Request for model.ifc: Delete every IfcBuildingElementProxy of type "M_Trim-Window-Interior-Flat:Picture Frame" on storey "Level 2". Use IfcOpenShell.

First a look at what the model holds.

```python
import ifcopenshell
import ifcopenshell.util.element

model = ifcopenshell.open("model.ifc")
print(model.schema)
storey = next(s for s in model.by_type("IfcBuildingStorey") if s.Name == "Level 2")
proxies = [e for e in ifcopenshell.util.element.get_decomposition(storey) if e.is_a("IfcBuildingElementProxy")]
seen = {}
for e in proxies:
    element_type = ifcopenshell.util.element.get_type(e)
    name = element_type.Name if element_type not in (None, e) else None
    seen[name] = seen.get(name, 0) + 1
for name, count in sorted(seen.items(), key=str):
    print(count, "x", name)
```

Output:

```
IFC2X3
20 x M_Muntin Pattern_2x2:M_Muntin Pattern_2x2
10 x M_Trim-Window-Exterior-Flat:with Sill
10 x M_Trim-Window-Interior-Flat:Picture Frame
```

```python
import ifcopenshell
import ifcopenshell.api.root
import ifcopenshell.util.element

model = ifcopenshell.open("model.ifc")

storey = next(s for s in model.by_type("IfcBuildingStorey") if s.Name == "Level 2")
proxies = [e for e in ifcopenshell.util.element.get_decomposition(storey) if e.is_a("IfcBuildingElementProxy")]
targets = [e for e in proxies if (t := ifcopenshell.util.element.get_type(e)) not in (None, e) and t.Name == "M_Trim-Window-Interior-Flat:Picture Frame"]

for e in targets:
    ifcopenshell.api.root.remove_product(model, product=e)
print(len(targets), "removed")

model.write("model_rev.ifc")
```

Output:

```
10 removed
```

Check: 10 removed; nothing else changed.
